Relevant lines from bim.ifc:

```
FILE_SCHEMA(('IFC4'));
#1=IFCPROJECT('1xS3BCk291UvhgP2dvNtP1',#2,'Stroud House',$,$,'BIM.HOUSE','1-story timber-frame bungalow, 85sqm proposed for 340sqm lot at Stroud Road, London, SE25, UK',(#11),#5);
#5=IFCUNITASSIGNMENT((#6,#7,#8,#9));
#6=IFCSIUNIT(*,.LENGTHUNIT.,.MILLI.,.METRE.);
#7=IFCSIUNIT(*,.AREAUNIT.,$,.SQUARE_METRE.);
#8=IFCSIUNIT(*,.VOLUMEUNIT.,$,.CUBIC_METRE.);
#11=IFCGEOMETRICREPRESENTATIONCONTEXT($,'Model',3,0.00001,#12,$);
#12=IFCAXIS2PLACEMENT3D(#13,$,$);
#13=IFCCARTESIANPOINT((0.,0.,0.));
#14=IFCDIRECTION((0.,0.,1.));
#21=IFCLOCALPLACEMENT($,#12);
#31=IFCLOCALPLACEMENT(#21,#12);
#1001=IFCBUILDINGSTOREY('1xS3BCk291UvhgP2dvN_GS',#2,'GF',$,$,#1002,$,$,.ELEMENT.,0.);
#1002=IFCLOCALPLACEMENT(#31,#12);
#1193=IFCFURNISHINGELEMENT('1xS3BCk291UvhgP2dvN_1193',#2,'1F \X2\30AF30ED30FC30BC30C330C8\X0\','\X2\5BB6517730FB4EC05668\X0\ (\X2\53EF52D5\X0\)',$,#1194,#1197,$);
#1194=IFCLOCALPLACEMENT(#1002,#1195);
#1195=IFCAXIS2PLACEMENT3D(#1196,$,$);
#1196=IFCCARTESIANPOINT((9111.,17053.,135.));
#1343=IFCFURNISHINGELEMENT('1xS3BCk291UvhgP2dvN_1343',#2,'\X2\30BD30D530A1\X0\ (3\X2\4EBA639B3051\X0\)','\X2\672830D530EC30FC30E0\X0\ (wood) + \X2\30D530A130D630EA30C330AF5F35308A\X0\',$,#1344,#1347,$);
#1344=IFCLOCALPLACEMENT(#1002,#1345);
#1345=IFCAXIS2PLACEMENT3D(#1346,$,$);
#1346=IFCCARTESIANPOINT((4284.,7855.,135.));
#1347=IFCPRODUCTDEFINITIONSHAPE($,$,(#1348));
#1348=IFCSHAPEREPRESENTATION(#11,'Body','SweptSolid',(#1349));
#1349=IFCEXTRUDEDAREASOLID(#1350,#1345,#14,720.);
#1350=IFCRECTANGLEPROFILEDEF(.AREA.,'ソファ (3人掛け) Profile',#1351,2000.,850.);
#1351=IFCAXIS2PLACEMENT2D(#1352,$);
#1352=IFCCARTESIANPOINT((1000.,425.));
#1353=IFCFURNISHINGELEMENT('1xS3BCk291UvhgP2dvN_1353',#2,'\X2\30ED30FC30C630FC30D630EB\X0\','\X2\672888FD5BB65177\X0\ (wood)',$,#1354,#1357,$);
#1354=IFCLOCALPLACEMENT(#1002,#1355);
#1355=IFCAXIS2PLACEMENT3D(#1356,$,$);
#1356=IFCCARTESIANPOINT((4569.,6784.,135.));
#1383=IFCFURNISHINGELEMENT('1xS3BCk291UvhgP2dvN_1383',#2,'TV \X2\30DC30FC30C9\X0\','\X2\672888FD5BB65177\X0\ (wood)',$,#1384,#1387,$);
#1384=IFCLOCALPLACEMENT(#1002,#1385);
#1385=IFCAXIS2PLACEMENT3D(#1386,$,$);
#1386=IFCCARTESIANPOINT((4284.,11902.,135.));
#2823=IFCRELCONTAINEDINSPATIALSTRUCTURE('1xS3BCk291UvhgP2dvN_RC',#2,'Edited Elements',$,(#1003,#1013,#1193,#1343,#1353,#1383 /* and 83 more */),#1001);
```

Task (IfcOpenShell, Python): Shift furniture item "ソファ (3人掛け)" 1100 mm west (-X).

```python
import ifcopenshell
import ifcopenshell.api.geometry
import ifcopenshell.util.placement
import ifcopenshell.util.unit

model = ifcopenshell.open("bim.ifc")
unit_scale = ifcopenshell.util.unit.calculate_unit_scale(model)

item = model.by_guid("1xS3BCk291UvhgP2dvN_1343")
matrix = ifcopenshell.util.placement.get_local_placement(item.ObjectPlacement)
matrix[0, 3] -= 1.1 / unit_scale
ifcopenshell.api.geometry.edit_object_placement(model, product=item, matrix=matrix, is_si=False)

print(ifcopenshell.util.placement.get_local_placement(item.ObjectPlacement).round(3) + 0.0)

model.write("bim-out.ifc")
```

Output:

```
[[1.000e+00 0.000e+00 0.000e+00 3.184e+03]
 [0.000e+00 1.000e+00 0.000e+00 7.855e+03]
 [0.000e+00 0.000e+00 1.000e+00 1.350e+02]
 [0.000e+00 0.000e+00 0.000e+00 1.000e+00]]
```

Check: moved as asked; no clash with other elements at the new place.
